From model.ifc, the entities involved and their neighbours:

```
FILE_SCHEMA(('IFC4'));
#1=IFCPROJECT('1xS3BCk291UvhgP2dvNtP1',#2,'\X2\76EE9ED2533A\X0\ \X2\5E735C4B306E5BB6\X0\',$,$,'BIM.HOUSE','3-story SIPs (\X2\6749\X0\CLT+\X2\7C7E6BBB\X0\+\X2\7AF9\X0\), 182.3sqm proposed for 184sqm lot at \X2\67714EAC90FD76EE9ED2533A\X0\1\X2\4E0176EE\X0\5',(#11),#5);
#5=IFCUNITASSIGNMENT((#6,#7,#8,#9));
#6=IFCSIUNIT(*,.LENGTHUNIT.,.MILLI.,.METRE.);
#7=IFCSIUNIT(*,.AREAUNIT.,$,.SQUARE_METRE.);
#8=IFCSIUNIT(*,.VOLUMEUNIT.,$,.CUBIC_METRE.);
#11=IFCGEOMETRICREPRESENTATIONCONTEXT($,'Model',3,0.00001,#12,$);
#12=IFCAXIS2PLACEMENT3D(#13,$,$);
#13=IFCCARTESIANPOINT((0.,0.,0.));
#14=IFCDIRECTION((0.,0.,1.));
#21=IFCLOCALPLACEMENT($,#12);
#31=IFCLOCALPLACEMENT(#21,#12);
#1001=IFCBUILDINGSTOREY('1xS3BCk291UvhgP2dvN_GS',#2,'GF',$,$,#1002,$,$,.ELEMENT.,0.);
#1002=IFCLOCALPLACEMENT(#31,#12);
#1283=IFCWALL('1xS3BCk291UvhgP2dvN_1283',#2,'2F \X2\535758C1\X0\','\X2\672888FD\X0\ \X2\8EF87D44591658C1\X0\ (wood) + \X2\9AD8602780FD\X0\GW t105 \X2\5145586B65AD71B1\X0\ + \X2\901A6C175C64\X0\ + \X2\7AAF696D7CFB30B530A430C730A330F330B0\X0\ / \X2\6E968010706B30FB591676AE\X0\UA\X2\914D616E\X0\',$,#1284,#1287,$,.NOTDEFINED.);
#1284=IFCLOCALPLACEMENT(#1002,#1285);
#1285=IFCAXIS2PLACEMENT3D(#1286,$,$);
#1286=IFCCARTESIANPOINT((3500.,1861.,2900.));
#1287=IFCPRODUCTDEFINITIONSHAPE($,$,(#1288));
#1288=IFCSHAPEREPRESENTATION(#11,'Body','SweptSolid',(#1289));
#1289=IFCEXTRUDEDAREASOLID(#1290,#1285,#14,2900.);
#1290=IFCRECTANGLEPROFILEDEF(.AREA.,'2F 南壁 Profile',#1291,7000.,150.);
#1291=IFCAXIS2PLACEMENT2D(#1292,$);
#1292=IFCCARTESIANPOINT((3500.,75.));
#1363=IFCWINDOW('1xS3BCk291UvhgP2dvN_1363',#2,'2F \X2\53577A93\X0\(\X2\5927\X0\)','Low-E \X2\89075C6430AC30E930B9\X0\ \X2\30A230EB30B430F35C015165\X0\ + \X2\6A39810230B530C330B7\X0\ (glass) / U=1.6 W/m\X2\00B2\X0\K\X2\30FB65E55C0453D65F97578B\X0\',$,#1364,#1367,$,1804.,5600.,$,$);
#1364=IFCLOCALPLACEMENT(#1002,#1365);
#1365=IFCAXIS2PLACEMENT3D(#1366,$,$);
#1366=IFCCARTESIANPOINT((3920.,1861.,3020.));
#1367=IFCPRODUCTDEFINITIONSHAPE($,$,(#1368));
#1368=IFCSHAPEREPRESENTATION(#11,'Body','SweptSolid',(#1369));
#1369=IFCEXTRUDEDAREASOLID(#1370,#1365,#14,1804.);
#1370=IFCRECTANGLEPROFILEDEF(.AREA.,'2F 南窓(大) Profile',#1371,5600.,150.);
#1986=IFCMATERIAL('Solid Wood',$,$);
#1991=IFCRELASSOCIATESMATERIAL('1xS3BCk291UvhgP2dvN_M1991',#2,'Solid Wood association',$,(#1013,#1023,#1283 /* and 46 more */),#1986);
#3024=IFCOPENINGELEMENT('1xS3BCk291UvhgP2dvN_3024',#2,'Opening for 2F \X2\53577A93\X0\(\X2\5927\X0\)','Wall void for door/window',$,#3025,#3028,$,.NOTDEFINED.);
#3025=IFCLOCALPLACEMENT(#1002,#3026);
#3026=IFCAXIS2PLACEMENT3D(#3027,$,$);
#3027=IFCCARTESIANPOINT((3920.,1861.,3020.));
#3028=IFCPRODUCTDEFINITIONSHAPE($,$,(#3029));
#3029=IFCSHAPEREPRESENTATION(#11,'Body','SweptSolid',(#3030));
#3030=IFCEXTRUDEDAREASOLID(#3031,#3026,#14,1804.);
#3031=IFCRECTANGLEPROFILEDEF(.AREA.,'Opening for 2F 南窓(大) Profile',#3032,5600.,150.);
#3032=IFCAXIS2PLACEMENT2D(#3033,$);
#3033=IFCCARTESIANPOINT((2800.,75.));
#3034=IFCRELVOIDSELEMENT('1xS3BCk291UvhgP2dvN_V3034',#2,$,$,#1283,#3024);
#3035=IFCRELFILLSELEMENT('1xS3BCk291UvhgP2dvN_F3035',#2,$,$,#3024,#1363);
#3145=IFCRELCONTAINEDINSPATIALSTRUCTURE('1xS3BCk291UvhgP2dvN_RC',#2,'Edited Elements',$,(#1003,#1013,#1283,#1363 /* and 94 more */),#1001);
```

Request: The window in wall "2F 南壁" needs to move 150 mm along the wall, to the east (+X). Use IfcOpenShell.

```python
import ifcopenshell
import ifcopenshell.api.geometry
import ifcopenshell.util.placement
import ifcopenshell.util.unit

model = ifcopenshell.open("model.ifc")
unit_scale = ifcopenshell.util.unit.calculate_unit_scale(model)

window = model.by_id(1363)
opening = window.FillsVoids[0].RelatingOpeningElement
wall = opening.VoidsElements[0].RelatingBuildingElement

wall_matrix = ifcopenshell.util.placement.get_local_placement(wall.ObjectPlacement)
shift = wall_matrix[:3, 0] * 0.15 / unit_scale
before = ifcopenshell.util.placement.get_local_placement(window.ObjectPlacement)[:3, 3].copy()

# The window is not placed relative to its opening, so move both.
for product in (opening, window):
    matrix = ifcopenshell.util.placement.get_local_placement(product.ObjectPlacement)
    matrix[:3, 3] += shift
    ifcopenshell.api.geometry.edit_object_placement(model, product=product, matrix=matrix, is_si=False)

after = ifcopenshell.util.placement.get_local_placement(window.ObjectPlacement)[:3, 3]
print("window moved by", (after - before).round(3) + 0.0)

model.write("model_edited.ifc")
```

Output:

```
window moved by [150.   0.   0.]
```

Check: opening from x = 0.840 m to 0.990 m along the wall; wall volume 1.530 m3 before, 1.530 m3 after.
